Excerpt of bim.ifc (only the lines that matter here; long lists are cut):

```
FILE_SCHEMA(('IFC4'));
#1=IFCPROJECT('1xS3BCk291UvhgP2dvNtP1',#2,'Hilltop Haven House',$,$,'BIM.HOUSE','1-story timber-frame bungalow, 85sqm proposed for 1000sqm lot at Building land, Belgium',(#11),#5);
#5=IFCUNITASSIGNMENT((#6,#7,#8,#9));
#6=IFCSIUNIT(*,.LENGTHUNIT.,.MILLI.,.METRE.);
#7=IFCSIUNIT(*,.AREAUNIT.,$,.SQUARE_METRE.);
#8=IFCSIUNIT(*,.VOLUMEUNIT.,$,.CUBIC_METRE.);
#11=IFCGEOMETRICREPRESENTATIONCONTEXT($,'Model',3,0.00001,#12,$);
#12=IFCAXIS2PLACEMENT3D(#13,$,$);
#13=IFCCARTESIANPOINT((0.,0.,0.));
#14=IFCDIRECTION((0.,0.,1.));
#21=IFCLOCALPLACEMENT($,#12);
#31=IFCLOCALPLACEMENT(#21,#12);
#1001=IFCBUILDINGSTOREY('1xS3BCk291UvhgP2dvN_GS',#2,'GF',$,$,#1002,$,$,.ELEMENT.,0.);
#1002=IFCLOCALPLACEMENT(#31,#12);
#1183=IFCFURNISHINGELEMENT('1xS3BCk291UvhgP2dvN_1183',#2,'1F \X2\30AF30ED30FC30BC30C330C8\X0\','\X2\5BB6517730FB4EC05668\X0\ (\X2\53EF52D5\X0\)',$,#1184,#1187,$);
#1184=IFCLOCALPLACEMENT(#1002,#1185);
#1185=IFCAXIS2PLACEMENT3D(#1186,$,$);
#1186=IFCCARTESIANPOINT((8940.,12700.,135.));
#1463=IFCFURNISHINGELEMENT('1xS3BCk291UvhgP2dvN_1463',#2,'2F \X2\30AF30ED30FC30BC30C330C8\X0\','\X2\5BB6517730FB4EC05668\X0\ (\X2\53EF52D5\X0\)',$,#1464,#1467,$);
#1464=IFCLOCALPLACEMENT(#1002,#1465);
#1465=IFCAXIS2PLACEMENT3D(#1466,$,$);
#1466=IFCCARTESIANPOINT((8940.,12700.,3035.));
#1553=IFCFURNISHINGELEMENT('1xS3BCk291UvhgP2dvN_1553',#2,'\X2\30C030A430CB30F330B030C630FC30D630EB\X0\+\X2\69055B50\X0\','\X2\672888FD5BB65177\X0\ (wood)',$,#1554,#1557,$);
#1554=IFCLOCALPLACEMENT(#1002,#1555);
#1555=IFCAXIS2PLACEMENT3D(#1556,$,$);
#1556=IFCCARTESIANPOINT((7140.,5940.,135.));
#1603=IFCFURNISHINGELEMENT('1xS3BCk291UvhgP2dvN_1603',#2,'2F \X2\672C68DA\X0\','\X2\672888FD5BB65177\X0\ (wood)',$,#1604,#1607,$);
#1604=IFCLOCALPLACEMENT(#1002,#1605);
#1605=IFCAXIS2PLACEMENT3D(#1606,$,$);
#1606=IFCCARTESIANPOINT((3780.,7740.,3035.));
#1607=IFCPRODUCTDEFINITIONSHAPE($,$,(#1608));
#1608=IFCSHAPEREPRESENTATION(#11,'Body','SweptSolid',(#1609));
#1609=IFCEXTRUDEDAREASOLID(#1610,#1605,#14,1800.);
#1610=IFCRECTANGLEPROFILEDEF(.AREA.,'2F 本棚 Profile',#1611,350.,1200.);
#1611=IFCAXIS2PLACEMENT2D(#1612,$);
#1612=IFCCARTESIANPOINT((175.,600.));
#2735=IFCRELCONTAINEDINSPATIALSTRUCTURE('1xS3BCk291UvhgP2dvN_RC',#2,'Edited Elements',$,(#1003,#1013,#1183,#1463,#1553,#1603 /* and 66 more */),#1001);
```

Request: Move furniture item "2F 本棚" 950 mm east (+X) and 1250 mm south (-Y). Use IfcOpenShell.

```python
import ifcopenshell
import ifcopenshell.api.geometry
import ifcopenshell.util.placement
import ifcopenshell.util.unit

model = ifcopenshell.open("bim.ifc")
unit_scale = ifcopenshell.util.unit.calculate_unit_scale(model)

item = model.by_id(1603)
matrix = ifcopenshell.util.placement.get_local_placement(item.ObjectPlacement)
matrix[0, 3] += 0.95 / unit_scale
matrix[1, 3] -= 1.25 / unit_scale
ifcopenshell.api.geometry.edit_object_placement(model, product=item, matrix=matrix, is_si=False)

print(ifcopenshell.util.placement.get_local_placement(item.ObjectPlacement).round(3) + 0.0)

model.write("bim-out.ifc")
```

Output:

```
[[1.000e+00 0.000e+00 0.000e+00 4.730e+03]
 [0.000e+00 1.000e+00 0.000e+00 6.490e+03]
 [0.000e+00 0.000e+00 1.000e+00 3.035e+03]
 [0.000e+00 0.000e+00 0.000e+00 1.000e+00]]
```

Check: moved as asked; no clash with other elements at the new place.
